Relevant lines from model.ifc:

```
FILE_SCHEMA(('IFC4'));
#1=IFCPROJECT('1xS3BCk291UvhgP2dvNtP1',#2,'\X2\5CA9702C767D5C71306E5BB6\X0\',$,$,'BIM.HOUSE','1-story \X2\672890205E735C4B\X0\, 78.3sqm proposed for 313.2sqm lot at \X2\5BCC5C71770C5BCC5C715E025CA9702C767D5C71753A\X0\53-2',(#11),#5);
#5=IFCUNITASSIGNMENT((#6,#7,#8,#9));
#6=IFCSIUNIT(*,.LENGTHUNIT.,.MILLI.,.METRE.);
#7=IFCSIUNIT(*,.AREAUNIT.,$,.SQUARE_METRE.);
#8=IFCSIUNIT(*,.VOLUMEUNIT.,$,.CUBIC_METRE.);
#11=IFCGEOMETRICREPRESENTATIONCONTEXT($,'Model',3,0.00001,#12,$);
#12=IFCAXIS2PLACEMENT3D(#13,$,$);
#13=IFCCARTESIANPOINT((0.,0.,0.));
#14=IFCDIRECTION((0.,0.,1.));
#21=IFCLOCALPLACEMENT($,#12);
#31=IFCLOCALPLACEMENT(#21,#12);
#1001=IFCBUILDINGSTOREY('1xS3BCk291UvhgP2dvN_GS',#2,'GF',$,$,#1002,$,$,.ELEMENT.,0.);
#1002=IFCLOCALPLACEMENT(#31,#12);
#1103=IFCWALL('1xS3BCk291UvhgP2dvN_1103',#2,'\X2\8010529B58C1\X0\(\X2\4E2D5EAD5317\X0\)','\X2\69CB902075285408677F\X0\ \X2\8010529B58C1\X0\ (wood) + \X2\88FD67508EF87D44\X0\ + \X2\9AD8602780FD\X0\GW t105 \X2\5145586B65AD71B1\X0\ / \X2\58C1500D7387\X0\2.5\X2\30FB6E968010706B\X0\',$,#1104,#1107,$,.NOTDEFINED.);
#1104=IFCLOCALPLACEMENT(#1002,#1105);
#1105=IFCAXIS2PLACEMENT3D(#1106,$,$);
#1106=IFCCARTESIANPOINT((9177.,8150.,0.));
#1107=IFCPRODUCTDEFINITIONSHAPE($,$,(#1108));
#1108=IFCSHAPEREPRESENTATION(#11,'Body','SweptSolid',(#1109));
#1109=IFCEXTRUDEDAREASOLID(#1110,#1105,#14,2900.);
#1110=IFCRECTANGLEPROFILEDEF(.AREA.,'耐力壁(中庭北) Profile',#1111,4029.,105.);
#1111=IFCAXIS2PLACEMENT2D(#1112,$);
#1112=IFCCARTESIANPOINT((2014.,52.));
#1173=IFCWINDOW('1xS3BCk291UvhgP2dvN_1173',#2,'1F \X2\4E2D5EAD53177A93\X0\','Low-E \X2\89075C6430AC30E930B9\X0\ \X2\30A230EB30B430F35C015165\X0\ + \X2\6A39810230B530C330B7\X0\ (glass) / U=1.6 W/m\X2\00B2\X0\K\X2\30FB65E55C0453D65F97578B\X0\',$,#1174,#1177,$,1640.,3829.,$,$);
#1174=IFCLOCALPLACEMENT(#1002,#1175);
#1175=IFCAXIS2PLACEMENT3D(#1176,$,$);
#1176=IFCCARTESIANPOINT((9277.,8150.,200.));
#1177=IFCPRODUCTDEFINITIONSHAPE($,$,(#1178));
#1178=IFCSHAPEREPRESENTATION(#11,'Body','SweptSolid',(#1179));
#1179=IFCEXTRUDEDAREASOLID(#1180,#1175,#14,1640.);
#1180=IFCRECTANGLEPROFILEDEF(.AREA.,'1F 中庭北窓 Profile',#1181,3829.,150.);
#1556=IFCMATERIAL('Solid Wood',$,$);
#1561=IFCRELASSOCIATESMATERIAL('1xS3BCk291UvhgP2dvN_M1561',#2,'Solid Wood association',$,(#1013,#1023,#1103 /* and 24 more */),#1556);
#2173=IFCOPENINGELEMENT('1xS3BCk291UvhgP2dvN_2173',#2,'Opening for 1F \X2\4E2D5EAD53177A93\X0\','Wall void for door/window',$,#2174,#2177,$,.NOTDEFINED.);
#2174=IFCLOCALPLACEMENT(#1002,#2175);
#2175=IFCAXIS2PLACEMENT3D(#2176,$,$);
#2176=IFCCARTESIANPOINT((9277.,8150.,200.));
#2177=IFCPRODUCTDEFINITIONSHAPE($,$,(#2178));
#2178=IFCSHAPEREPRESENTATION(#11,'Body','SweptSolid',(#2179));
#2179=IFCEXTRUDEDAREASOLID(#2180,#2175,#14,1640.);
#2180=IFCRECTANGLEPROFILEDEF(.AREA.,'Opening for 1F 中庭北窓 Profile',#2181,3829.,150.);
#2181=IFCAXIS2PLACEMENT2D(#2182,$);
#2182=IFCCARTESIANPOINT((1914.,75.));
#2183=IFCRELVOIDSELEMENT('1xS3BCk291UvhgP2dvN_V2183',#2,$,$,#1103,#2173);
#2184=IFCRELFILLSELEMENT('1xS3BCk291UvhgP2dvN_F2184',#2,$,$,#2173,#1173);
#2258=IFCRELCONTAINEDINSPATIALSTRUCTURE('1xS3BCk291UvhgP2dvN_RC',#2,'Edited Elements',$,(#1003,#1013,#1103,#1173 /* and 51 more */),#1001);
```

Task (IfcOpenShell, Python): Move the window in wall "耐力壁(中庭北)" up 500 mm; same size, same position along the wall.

```python
import numpy as np
import ifcopenshell
import ifcopenshell.api.geometry
import ifcopenshell.util.placement
import ifcopenshell.util.unit

model = ifcopenshell.open("model.ifc")
unit_scale = ifcopenshell.util.unit.calculate_unit_scale(model)

window = model.by_guid("1xS3BCk291UvhgP2dvN_1173")
opening = window.FillsVoids[0].RelatingOpeningElement
dz = 0.5 / unit_scale

shift = np.array([0.0, 0.0, dz])
# The window is not placed relative to its opening, so move both.
for product in (opening, window):
    matrix = ifcopenshell.util.placement.get_local_placement(product.ObjectPlacement)
    matrix[:3, 3] += shift
    ifcopenshell.api.geometry.edit_object_placement(model, product=product, matrix=matrix, is_si=False)

print(f"moved by {dz * unit_scale:+.3f} m")

model.write("model_v2.ifc")
```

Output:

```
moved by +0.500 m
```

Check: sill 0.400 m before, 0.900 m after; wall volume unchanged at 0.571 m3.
